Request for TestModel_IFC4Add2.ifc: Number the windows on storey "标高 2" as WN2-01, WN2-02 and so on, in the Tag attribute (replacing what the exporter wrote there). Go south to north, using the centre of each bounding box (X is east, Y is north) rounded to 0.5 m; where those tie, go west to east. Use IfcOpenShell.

First a look at what the model holds.

```python
import ifcopenshell
import ifcopenshell.util.element
import ifcopenshell.util.placement

model = ifcopenshell.open("TestModel_IFC4Add2.ifc")
print(model.schema)
storey = next(s for s in model.by_type("IfcBuildingStorey") if s.Name == "标高 2")
windows = [e for e in ifcopenshell.util.element.get_decomposition(storey) if e.is_a("IfcWindow")]
for e in sorted(windows, key=lambda e: e.id()):
    origin = ifcopenshell.util.placement.get_local_placement(e.ObjectPlacement)[:3, 3]
    print(e.id(), e.Tag, e.Name, origin.round(2) + 0.0, sep=" | ")
```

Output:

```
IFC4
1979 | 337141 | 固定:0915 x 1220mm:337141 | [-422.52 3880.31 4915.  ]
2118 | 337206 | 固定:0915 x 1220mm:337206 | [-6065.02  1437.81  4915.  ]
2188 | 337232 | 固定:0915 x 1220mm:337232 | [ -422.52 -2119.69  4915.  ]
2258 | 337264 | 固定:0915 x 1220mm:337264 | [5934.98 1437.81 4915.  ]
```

```python
import ifcopenshell
import ifcopenshell.geom
import ifcopenshell.util.element
import ifcopenshell.util.shape

model = ifcopenshell.open("TestModel_IFC4Add2.ifc")
settings = ifcopenshell.geom.settings()
settings.set("use-world-coords", True)


def centre(element):
    shape = ifcopenshell.geom.create_shape(settings, element)
    return ifcopenshell.util.shape.get_bbox_centroid(shape.geometry)


storey = next(s for s in model.by_type("IfcBuildingStorey") if s.Name == "标高 2")
windows = [e for e in ifcopenshell.util.element.get_decomposition(storey) if e.is_a("IfcWindow")]

# Insertion points can sit at a corner or the storey origin, so sort by the geometry (in metres).
centres = {e: centre(e) for e in windows}
windows.sort(key=lambda e: (round(centres[e][1] / 0.5), centres[e][0]))

for i, e in enumerate(windows, start=1):
    number = f"WN2-{i:02d}"
    e.Tag = number
    print(e.id(), number)

model.write("TestModel_IFC4Add2-out.ifc")
```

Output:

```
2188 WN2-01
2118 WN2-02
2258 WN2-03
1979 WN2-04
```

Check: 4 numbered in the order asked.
